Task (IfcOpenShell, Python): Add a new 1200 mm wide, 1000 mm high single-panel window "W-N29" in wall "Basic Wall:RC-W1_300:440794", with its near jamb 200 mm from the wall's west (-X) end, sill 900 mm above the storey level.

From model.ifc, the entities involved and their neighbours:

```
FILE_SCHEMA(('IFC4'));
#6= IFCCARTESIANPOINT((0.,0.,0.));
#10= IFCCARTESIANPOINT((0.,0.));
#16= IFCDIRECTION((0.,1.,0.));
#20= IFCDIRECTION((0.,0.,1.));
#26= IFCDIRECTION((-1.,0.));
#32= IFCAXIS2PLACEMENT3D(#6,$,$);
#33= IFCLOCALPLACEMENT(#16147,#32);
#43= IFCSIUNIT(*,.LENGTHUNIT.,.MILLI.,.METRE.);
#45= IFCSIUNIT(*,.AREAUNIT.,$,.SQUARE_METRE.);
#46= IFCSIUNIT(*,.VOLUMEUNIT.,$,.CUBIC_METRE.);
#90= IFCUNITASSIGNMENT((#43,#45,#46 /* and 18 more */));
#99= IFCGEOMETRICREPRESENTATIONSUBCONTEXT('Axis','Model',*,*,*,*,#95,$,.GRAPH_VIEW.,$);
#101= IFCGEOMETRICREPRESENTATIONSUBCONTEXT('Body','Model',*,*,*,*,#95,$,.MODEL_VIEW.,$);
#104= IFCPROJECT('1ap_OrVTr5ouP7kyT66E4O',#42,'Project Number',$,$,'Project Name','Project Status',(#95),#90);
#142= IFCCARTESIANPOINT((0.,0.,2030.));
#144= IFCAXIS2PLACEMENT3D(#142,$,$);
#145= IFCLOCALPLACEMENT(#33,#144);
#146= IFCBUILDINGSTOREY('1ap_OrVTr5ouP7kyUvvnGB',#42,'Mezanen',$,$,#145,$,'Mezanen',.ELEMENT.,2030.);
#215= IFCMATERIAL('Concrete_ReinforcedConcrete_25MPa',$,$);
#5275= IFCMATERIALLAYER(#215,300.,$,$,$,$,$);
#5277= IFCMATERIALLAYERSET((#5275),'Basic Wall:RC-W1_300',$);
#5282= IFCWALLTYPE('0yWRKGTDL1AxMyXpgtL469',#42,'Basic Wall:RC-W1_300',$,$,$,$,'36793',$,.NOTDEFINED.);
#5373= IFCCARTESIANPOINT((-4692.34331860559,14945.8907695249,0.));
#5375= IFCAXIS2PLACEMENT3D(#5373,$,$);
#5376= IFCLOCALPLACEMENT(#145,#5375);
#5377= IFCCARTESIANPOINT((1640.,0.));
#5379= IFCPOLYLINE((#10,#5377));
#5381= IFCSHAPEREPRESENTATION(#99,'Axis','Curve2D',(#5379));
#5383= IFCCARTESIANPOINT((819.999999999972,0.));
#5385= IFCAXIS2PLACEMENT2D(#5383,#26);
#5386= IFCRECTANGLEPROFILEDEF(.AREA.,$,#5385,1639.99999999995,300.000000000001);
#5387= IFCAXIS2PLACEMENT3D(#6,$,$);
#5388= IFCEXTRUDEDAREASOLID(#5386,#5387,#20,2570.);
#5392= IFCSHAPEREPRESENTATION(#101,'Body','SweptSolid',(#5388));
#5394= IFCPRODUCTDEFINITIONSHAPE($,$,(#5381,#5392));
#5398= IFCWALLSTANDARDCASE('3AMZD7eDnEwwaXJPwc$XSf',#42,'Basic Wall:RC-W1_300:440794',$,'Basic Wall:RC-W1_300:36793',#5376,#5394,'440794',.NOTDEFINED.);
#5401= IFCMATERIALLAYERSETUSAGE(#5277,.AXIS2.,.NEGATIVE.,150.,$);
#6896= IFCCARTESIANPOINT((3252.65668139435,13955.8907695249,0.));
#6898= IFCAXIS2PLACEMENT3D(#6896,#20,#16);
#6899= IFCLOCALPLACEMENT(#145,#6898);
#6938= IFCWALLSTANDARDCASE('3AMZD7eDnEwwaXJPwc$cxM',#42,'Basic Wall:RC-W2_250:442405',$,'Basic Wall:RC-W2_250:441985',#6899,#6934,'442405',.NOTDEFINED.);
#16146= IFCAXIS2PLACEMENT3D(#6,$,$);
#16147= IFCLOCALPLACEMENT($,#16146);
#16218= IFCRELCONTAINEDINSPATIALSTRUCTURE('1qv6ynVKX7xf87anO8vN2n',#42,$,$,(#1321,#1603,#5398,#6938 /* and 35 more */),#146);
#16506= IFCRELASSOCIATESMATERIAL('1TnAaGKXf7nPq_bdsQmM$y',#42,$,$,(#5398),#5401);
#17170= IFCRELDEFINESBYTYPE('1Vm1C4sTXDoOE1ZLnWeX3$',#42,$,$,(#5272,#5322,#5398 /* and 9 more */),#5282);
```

```python
import numpy as np
import ifcopenshell
import ifcopenshell.api.feature
import ifcopenshell.api.geometry
import ifcopenshell.api.root
import ifcopenshell.api.spatial
import ifcopenshell.geom
import ifcopenshell.util.element
import ifcopenshell.util.placement
import ifcopenshell.util.representation
import ifcopenshell.util.shape
import ifcopenshell.util.unit

model = ifcopenshell.open("model.ifc")
unit_scale = ifcopenshell.util.unit.calculate_unit_scale(model)
settings = ifcopenshell.geom.settings()


def volume(element):
    """Net volume in cubic metres, openings subtracted."""
    shape = ifcopenshell.geom.create_shape(settings, element)
    return ifcopenshell.util.shape.get_volume(shape.geometry)


wall = model.by_id(5398)
storey = ifcopenshell.util.element.get_container(wall, ifc_class="IfcBuildingStorey")
context = ifcopenshell.util.representation.get_context(model, "Model", "Body", "MODEL_VIEW")
before = volume(wall)

width, height, from_end, sill = 1.2, 1, 0.2, 0.9  # metres

# The wall runs along its own X axis, and the end named is its -X end.
wall_shape = ifcopenshell.geom.create_shape(settings, wall)
x, y, z = ifcopenshell.util.shape.get_vertices(wall_shape.geometry).T
start = x.min() + from_end
face, thickness = float(y.min()), float(y.max() - y.min())
wall_matrix = ifcopenshell.util.placement.get_local_placement(wall.ObjectPlacement)
level = ifcopenshell.util.placement.get_local_placement(storey.ObjectPlacement)[2, 3]


def in_wall(x, y):
    """Placement at x, y metres in the wall's axes, at sill height."""
    matrix = wall_matrix.copy()
    matrix[:, 3] = wall_matrix @ np.array([x / unit_scale, y / unit_scale, 0.0, 1.0])
    matrix[2, 3] = level + sill / unit_scale
    return matrix


# Opening: a box that overshoots both wall faces by 50 mm.
opening = ifcopenshell.api.root.create_entity(model, ifc_class="IfcOpeningElement", predefined_type="OPENING")
box = ifcopenshell.api.geometry.add_wall_representation(
    model, context=context, length=width, height=height, thickness=thickness + 0.1
)
ifcopenshell.api.geometry.assign_representation(model, product=opening, representation=box)
ifcopenshell.api.geometry.edit_object_placement(model, product=opening, matrix=in_wall(start, face - 0.05), is_si=False)
ifcopenshell.api.feature.add_feature(model, feature=opening, element=wall)

window = ifcopenshell.api.root.create_entity(model, ifc_class="IfcWindow", name="W-N29", predefined_type="WINDOW")
window.OverallWidth, window.OverallHeight = width / unit_scale, height / unit_scale
window.PartitioningType = "SINGLE_PANEL"
body = ifcopenshell.api.geometry.add_window_representation(
    model,
    context=context,
    overall_width=window.OverallWidth,
    overall_height=window.OverallHeight,
    partition_type="SINGLE_PANEL",
)
ifcopenshell.api.geometry.assign_representation(model, product=window, representation=body)
ifcopenshell.api.spatial.assign_container(model, products=[window], relating_structure=storey)
ifcopenshell.api.feature.add_filling(model, opening=opening, element=window)

# Centre the window in the wall's thickness.
ifcopenshell.api.geometry.edit_object_placement(model, product=window, matrix=in_wall(start, face), is_si=False)
window_shape = ifcopenshell.geom.create_shape(settings, window)
depth = ifcopenshell.util.shape.get_vertices(window_shape.geometry)[:, 1]
offset = face + thickness / 2 - (depth.min() + depth.max()) / 2
ifcopenshell.api.geometry.edit_object_placement(model, product=window, matrix=in_wall(start, offset), is_si=False)

after = volume(wall)

print(f"wall volume {before:.3f} -> {after:.3f} m3")

model.write("model-out.ifc")
```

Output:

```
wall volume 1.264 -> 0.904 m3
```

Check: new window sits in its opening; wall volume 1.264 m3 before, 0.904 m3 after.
